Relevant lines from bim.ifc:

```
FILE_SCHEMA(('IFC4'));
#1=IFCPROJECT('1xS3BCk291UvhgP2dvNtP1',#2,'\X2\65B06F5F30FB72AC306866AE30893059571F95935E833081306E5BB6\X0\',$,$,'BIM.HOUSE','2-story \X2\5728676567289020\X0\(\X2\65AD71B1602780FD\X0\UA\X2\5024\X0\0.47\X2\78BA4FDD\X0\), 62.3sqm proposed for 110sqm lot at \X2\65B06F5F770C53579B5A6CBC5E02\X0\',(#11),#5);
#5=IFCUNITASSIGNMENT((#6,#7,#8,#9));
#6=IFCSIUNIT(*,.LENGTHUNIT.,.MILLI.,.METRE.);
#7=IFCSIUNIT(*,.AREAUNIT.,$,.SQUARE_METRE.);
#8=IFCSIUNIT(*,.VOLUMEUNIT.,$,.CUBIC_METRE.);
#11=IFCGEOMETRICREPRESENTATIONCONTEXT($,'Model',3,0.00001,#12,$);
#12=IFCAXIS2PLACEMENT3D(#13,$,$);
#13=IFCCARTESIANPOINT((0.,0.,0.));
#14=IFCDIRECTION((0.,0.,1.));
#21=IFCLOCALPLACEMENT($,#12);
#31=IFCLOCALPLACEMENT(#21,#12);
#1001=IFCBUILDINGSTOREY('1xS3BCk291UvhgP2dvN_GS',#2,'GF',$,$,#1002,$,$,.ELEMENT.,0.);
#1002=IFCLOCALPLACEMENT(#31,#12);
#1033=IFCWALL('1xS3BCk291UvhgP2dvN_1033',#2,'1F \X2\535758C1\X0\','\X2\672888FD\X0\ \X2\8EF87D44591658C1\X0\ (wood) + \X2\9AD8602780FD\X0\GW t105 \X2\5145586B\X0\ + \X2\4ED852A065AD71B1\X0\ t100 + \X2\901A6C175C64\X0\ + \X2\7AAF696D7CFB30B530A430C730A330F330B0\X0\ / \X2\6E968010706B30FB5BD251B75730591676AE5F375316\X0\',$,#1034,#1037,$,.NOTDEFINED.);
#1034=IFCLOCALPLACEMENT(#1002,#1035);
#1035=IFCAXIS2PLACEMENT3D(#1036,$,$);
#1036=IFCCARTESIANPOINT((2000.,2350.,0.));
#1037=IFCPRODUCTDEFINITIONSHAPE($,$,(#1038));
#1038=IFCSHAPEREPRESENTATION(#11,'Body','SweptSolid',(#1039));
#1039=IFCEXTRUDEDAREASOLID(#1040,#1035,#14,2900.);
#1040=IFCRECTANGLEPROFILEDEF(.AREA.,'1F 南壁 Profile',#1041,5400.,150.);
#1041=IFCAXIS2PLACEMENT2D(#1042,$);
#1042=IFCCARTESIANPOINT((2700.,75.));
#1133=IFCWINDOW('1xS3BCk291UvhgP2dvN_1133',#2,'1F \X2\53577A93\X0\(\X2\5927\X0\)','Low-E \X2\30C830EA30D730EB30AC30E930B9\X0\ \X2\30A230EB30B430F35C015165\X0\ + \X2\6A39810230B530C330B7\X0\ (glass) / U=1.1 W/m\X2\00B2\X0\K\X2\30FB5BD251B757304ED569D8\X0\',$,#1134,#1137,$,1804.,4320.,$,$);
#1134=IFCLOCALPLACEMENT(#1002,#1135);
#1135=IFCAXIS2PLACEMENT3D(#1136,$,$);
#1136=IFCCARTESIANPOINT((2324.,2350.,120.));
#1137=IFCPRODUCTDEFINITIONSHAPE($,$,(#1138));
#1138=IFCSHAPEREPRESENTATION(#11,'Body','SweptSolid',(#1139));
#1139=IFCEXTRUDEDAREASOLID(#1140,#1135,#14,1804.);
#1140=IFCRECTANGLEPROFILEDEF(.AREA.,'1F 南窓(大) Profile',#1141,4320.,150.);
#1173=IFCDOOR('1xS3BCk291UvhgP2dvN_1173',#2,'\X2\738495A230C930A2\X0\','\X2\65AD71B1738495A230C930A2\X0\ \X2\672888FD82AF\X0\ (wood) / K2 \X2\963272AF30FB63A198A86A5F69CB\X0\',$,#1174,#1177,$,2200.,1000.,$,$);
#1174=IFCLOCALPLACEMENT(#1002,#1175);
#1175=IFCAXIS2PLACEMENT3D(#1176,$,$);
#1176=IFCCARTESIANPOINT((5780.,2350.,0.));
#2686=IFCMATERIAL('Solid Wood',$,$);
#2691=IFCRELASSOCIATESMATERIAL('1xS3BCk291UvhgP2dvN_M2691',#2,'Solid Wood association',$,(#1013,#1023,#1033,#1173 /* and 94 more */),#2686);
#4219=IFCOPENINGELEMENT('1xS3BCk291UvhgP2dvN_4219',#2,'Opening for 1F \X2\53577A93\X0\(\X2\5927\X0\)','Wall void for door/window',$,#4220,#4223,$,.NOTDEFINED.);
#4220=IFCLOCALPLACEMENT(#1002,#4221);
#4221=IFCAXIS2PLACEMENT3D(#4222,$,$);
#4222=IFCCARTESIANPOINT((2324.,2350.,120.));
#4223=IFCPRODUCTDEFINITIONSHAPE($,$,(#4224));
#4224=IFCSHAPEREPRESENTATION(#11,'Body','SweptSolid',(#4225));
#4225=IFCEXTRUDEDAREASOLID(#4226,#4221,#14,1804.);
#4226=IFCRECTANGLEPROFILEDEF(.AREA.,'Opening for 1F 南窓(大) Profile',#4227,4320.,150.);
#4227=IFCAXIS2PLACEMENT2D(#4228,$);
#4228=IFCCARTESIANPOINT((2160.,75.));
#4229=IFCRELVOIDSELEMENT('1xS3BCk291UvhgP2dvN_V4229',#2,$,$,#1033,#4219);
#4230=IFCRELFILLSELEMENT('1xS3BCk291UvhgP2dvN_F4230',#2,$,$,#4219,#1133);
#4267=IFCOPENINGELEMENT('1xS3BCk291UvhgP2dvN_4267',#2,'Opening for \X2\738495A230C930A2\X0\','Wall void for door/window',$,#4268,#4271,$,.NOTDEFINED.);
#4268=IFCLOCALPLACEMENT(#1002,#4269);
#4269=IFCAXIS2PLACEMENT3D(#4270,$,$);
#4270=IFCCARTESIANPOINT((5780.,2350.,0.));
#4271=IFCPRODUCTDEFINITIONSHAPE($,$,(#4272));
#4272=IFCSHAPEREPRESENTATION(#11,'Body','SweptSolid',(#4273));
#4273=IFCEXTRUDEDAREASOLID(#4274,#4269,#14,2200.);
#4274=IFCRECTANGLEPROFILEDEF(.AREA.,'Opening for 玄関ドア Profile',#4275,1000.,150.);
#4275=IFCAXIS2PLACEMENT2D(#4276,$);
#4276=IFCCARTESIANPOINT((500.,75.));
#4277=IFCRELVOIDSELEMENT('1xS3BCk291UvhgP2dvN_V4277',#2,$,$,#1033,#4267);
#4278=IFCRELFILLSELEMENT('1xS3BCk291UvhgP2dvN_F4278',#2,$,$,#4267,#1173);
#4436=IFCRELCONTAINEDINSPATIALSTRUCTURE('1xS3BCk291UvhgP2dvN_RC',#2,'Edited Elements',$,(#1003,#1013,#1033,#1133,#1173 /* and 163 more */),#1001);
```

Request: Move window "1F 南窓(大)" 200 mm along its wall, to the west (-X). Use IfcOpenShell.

```python
import ifcopenshell
import ifcopenshell.api.geometry
import ifcopenshell.util.placement
import ifcopenshell.util.unit

model = ifcopenshell.open("bim.ifc")
unit_scale = ifcopenshell.util.unit.calculate_unit_scale(model)

window = model.by_id(1133)
opening = window.FillsVoids[0].RelatingOpeningElement
wall = opening.VoidsElements[0].RelatingBuildingElement

wall_matrix = ifcopenshell.util.placement.get_local_placement(wall.ObjectPlacement)
shift = wall_matrix[:3, 0] * -0.2 / unit_scale
before = ifcopenshell.util.placement.get_local_placement(window.ObjectPlacement)[:3, 3].copy()

# The window is not placed relative to its opening, so move both.
for product in (opening, window):
    matrix = ifcopenshell.util.placement.get_local_placement(product.ObjectPlacement)
    matrix[:3, 3] += shift
    ifcopenshell.api.geometry.edit_object_placement(model, product=product, matrix=matrix, is_si=False)

after = ifcopenshell.util.placement.get_local_placement(window.ObjectPlacement)[:3, 3]
print("window moved by", (after - before).round(3) + 0.0)

model.write("bim_v2.ifc")
```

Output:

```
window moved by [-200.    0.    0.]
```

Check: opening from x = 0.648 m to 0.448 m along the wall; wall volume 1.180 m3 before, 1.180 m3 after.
